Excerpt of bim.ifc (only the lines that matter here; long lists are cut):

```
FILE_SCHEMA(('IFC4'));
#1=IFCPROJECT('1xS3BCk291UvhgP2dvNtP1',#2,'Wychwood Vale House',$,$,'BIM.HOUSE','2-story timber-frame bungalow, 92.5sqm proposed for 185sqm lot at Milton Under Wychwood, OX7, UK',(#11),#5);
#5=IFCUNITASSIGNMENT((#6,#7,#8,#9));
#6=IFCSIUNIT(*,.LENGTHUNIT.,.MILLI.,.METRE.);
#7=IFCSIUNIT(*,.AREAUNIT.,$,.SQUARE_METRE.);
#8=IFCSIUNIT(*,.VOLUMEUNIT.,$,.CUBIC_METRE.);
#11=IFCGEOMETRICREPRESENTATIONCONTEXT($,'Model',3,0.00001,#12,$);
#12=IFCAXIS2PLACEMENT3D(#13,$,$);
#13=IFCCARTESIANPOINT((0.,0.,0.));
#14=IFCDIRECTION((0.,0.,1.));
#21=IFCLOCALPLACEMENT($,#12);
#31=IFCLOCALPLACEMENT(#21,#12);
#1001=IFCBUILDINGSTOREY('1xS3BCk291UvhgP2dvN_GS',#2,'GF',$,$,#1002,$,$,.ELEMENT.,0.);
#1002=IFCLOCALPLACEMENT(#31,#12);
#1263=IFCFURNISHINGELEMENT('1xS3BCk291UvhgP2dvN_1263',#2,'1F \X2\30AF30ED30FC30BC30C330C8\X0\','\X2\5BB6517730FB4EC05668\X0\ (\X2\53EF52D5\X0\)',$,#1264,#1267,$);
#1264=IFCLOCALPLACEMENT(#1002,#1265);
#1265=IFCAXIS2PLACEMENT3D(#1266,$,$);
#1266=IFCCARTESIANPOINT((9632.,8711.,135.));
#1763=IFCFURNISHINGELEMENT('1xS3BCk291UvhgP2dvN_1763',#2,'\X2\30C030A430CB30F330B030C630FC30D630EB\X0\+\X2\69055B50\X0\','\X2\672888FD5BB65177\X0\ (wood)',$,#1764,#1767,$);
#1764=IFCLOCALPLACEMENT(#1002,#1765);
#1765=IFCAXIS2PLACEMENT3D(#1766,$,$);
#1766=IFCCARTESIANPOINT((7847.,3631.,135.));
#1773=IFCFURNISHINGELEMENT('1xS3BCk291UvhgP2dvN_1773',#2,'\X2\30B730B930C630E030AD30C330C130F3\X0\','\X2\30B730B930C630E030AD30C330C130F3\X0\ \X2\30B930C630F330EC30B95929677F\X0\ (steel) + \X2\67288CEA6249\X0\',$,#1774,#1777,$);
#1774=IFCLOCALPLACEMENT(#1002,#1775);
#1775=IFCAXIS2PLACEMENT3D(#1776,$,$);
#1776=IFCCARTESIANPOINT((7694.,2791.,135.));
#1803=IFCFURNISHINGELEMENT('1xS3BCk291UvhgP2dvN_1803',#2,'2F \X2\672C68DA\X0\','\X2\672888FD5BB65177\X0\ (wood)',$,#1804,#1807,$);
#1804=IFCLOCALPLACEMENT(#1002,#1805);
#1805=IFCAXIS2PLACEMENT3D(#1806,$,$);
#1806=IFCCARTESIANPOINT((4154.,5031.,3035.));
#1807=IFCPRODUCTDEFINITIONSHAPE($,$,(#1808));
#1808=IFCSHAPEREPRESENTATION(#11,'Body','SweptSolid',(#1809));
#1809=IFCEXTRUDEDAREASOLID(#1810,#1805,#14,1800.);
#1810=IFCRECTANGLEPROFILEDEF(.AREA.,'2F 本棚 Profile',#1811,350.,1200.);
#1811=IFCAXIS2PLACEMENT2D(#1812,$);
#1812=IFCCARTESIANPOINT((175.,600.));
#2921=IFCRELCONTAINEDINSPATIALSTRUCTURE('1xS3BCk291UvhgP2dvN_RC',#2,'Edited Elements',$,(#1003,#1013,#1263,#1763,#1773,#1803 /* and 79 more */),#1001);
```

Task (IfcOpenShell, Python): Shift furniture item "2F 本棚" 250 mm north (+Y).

```python
import ifcopenshell
import ifcopenshell.api.geometry
import ifcopenshell.util.placement

model = ifcopenshell.open("bim.ifc")

item = model.by_guid("1xS3BCk291UvhgP2dvN_1803")
matrix = ifcopenshell.util.placement.get_local_placement(item.ObjectPlacement)
matrix[1, 3] += 250.0
ifcopenshell.api.geometry.edit_object_placement(model, product=item, matrix=matrix, is_si=False)

print(ifcopenshell.util.placement.get_local_placement(item.ObjectPlacement).round(3) + 0.0)

model.write("bim_rev.ifc")
```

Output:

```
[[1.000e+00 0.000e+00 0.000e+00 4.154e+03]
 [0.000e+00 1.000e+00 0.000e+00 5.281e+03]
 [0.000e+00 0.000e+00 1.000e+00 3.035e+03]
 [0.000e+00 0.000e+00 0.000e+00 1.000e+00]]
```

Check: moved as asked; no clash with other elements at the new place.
